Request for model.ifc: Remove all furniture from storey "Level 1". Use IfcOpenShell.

First a look at what the model holds.

```python
import ifcopenshell
import ifcopenshell.util.element

model = ifcopenshell.open("model.ifc")
print(model.schema)
storey = next(s for s in model.by_type("IfcBuildingStorey") if s.Name == "Level 1")
furniture = [e for e in ifcopenshell.util.element.get_decomposition(storey) if e.is_a("IfcFurnishingElement")]
seen = {}
for e in furniture:
    element_type = ifcopenshell.util.element.get_type(e)
    name = element_type.Name if element_type not in (None, e) else None
    seen[name] = seen.get(name, 0) + 1
for name, count in sorted(seen.items(), key=str):
    print(count, "x", name)
```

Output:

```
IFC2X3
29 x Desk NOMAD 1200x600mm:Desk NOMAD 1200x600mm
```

```python
import ifcopenshell
import ifcopenshell.api.root
import ifcopenshell.util.element

model = ifcopenshell.open("model.ifc")

storey = next(s for s in model.by_type("IfcBuildingStorey") if s.Name == "Level 1")
furniture = [e for e in ifcopenshell.util.element.get_decomposition(storey) if e.is_a("IfcFurnishingElement")]

for e in furniture:
    ifcopenshell.api.root.remove_product(model, product=e)
print(len(furniture), "removed")

model.write("model_rev.ifc")
```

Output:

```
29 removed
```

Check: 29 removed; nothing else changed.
